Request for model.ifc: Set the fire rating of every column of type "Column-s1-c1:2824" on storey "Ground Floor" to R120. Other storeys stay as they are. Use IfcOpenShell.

First a look at what the model holds.

```python
import ifcopenshell
import ifcopenshell.util.element

model = ifcopenshell.open("model.ifc")
print(model.schema)
storey = next(s for s in model.by_type("IfcBuildingStorey") if s.Name == "Ground Floor")
columns = [e for e in ifcopenshell.util.element.get_decomposition(storey) if e.is_a("IfcColumn")]
seen = {}
for e in columns:
    element_type = ifcopenshell.util.element.get_type(e)
    key = (element_type.Name if element_type != e and element_type else None, ifcopenshell.util.element.get_pset(e, "Pset_ColumnCommon", "FireRating"))
    seen[key] = seen.get(key, 0) + 1
for (name, value), count in sorted(seen.items(), key=str):
    print(count, "x", name, "|", value)
```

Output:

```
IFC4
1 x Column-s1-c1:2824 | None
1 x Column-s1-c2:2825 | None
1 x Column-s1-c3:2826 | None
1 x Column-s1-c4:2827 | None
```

```python
import ifcopenshell
import ifcopenshell.api.pset
import ifcopenshell.util.element

model = ifcopenshell.open("model.ifc")

storey = next(s for s in model.by_type("IfcBuildingStorey") if s.Name == "Ground Floor")
columns = [e for e in ifcopenshell.util.element.get_decomposition(storey) if e.is_a("IfcColumn")]

count = 0
for e in columns:
    element_type = ifcopenshell.util.element.get_type(e)
    if element_type in (None, e) or element_type.Name != "Column-s1-c1:2824":
        continue
    # add_pset returns the element's existing set when there is one.
    pset = ifcopenshell.api.pset.add_pset(model, product=e, name="Pset_ColumnCommon")
    ifcopenshell.api.pset.edit_pset(model, pset=pset, properties={"FireRating": "R120"})
    count += 1

print(count, "columns updated")

model.write("model_updated.ifc")
```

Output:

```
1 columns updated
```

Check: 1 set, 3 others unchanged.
